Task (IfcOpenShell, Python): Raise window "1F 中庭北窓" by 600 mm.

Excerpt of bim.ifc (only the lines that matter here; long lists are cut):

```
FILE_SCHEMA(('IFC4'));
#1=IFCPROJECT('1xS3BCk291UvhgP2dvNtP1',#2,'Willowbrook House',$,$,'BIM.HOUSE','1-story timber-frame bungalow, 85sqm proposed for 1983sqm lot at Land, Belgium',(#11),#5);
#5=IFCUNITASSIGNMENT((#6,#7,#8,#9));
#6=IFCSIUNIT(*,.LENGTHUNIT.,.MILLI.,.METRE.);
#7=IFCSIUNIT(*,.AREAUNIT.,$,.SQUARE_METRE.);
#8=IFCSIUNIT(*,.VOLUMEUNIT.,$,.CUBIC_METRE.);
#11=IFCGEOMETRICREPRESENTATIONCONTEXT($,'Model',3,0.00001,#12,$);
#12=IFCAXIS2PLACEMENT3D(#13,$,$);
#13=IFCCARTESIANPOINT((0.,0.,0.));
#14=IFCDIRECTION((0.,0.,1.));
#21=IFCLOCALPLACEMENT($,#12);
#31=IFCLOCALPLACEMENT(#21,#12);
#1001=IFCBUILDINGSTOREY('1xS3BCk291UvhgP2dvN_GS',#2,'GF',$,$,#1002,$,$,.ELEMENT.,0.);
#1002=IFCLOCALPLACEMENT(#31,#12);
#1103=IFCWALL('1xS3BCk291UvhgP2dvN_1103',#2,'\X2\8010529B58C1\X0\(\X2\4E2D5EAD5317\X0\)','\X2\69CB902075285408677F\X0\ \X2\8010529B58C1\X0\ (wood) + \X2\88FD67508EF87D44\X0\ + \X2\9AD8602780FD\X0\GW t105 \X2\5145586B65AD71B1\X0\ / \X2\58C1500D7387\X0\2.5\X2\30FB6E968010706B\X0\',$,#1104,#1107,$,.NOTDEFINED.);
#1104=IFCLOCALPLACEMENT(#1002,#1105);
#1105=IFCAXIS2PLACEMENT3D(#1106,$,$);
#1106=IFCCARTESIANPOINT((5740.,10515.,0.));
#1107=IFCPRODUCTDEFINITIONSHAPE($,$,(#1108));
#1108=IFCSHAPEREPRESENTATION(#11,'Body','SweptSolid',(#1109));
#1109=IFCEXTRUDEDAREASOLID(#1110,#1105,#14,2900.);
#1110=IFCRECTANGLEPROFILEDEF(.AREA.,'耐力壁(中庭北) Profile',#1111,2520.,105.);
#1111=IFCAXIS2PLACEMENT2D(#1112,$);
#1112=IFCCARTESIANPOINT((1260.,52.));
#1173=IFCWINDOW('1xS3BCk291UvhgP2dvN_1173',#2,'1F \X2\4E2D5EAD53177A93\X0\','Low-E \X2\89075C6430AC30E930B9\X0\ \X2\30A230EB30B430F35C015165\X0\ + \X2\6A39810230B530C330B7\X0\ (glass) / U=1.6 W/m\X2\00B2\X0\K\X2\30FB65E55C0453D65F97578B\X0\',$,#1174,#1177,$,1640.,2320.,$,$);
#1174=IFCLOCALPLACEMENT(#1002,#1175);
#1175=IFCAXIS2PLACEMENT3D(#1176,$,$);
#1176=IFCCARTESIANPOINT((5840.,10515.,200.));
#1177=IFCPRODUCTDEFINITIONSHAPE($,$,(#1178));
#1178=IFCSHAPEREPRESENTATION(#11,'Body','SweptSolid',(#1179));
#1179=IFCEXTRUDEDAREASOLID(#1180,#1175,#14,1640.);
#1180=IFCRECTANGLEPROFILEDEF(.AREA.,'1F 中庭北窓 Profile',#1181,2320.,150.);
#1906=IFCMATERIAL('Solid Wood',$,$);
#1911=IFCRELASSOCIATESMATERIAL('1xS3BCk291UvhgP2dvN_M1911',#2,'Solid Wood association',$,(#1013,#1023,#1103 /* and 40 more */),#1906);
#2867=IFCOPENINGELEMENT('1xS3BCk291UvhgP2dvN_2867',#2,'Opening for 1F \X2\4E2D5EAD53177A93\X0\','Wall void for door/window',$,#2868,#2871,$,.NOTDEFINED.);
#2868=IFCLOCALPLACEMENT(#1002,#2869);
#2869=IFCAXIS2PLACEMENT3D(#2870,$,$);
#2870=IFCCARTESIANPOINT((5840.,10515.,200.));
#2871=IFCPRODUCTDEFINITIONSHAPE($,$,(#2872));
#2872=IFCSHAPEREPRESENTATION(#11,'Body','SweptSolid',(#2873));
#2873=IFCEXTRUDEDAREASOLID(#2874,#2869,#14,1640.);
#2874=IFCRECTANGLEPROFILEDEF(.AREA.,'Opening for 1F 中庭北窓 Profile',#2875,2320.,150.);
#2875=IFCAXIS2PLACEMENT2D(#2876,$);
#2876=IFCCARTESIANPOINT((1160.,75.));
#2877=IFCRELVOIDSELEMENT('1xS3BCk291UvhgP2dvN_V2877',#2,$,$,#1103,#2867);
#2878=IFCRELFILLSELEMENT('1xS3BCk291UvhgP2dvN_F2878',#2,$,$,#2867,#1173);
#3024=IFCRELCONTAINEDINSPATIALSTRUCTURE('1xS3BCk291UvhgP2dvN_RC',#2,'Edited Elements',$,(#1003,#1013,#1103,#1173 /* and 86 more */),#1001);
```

```python
import numpy as np
import ifcopenshell
import ifcopenshell.api.geometry
import ifcopenshell.util.placement
import ifcopenshell.util.unit

model = ifcopenshell.open("bim.ifc")
unit_scale = ifcopenshell.util.unit.calculate_unit_scale(model)

window = model.by_id(1173)
opening = window.FillsVoids[0].RelatingOpeningElement
dz = 0.6 / unit_scale

shift = np.array([0.0, 0.0, dz])
# The window is not placed relative to its opening, so move both.
for product in (opening, window):
    matrix = ifcopenshell.util.placement.get_local_placement(product.ObjectPlacement)
    matrix[:3, 3] += shift
    ifcopenshell.api.geometry.edit_object_placement(model, product=product, matrix=matrix, is_si=False)

print(f"moved by {dz * unit_scale:+.3f} m")

model.write("bim_rev.ifc")
```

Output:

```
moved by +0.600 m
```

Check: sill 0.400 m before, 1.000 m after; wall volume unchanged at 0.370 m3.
